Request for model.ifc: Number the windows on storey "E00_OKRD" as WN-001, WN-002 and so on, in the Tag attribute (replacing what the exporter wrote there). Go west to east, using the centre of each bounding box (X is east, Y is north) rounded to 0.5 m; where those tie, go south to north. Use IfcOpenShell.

First a look at what the model holds.

```python
import ifcopenshell
import ifcopenshell.util.element
import ifcopenshell.util.placement

model = ifcopenshell.open("model.ifc")
print(model.schema)
storey = next(s for s in model.by_type("IfcBuildingStorey") if s.Name == "E00_OKRD")
windows = [e for e in ifcopenshell.util.element.get_decomposition(storey) if e.is_a("IfcWindow")]
for e in sorted(windows, key=lambda e: e.id()):
    origin = ifcopenshell.util.placement.get_local_placement(e.ObjectPlacement)[:3, 3]
    print(e.id(), e.Tag, e.Name, origin.round(2) + 0.0, sep=" | ")
```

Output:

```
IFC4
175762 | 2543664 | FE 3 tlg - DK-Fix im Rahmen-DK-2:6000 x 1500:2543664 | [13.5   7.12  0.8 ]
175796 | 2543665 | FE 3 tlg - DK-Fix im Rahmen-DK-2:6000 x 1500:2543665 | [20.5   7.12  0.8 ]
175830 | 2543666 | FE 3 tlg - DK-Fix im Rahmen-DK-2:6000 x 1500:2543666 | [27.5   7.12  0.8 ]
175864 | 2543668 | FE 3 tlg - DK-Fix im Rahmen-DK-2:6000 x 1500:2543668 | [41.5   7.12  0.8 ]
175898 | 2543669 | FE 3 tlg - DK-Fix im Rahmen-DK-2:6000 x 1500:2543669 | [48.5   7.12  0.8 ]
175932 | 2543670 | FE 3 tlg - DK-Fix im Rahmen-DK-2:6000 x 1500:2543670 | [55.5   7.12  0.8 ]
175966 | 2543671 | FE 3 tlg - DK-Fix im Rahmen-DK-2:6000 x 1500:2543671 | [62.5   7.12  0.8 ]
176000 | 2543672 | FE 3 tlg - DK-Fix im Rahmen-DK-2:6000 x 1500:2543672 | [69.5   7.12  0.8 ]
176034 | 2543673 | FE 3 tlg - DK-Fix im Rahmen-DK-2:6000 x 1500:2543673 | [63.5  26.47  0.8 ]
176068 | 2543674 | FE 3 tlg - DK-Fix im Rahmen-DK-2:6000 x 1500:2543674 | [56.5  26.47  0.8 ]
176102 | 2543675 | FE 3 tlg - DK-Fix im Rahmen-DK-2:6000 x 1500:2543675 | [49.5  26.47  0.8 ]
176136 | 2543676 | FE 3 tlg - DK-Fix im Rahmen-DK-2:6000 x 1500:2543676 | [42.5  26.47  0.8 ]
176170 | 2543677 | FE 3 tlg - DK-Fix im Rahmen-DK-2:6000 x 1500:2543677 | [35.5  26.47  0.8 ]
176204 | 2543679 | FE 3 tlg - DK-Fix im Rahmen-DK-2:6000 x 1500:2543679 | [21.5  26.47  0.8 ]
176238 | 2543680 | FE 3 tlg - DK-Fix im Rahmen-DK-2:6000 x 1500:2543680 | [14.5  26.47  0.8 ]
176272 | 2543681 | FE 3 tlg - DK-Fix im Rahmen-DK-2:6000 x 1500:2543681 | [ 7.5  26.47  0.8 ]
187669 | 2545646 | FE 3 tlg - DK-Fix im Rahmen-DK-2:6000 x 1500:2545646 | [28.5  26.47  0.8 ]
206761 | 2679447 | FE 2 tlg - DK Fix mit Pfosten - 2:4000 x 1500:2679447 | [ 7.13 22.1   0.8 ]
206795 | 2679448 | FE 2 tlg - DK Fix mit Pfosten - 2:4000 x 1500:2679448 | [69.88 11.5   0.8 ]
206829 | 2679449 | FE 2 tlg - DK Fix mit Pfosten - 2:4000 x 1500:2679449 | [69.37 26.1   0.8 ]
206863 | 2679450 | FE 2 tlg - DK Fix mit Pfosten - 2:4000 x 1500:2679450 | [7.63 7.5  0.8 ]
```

```python
import ifcopenshell
import ifcopenshell.geom
import ifcopenshell.util.element
import ifcopenshell.util.shape

model = ifcopenshell.open("model.ifc")
settings = ifcopenshell.geom.settings()
settings.set("use-world-coords", True)


def centre(element):
    shape = ifcopenshell.geom.create_shape(settings, element)
    return ifcopenshell.util.shape.get_bbox_centroid(shape.geometry)


storey = next(s for s in model.by_type("IfcBuildingStorey") if s.Name == "E00_OKRD")
windows = [e for e in ifcopenshell.util.element.get_decomposition(storey) if e.is_a("IfcWindow")]

# Insertion points can sit at a corner or the storey origin, so sort by the geometry (in metres).
centres = {e: centre(e) for e in windows}
windows.sort(key=lambda e: (round(centres[e][0] / 0.5), centres[e][1]))

for i, e in enumerate(windows, start=1):
    number = f"WN-0{i:02d}"
    e.Tag = number
    print(e.id(), number)

model.write("model_updated.ifc")
```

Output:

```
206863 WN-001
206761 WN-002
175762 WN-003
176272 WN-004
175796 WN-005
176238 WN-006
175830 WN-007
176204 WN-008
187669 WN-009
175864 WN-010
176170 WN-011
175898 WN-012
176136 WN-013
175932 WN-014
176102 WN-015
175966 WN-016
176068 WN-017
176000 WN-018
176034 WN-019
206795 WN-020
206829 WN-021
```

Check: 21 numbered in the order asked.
